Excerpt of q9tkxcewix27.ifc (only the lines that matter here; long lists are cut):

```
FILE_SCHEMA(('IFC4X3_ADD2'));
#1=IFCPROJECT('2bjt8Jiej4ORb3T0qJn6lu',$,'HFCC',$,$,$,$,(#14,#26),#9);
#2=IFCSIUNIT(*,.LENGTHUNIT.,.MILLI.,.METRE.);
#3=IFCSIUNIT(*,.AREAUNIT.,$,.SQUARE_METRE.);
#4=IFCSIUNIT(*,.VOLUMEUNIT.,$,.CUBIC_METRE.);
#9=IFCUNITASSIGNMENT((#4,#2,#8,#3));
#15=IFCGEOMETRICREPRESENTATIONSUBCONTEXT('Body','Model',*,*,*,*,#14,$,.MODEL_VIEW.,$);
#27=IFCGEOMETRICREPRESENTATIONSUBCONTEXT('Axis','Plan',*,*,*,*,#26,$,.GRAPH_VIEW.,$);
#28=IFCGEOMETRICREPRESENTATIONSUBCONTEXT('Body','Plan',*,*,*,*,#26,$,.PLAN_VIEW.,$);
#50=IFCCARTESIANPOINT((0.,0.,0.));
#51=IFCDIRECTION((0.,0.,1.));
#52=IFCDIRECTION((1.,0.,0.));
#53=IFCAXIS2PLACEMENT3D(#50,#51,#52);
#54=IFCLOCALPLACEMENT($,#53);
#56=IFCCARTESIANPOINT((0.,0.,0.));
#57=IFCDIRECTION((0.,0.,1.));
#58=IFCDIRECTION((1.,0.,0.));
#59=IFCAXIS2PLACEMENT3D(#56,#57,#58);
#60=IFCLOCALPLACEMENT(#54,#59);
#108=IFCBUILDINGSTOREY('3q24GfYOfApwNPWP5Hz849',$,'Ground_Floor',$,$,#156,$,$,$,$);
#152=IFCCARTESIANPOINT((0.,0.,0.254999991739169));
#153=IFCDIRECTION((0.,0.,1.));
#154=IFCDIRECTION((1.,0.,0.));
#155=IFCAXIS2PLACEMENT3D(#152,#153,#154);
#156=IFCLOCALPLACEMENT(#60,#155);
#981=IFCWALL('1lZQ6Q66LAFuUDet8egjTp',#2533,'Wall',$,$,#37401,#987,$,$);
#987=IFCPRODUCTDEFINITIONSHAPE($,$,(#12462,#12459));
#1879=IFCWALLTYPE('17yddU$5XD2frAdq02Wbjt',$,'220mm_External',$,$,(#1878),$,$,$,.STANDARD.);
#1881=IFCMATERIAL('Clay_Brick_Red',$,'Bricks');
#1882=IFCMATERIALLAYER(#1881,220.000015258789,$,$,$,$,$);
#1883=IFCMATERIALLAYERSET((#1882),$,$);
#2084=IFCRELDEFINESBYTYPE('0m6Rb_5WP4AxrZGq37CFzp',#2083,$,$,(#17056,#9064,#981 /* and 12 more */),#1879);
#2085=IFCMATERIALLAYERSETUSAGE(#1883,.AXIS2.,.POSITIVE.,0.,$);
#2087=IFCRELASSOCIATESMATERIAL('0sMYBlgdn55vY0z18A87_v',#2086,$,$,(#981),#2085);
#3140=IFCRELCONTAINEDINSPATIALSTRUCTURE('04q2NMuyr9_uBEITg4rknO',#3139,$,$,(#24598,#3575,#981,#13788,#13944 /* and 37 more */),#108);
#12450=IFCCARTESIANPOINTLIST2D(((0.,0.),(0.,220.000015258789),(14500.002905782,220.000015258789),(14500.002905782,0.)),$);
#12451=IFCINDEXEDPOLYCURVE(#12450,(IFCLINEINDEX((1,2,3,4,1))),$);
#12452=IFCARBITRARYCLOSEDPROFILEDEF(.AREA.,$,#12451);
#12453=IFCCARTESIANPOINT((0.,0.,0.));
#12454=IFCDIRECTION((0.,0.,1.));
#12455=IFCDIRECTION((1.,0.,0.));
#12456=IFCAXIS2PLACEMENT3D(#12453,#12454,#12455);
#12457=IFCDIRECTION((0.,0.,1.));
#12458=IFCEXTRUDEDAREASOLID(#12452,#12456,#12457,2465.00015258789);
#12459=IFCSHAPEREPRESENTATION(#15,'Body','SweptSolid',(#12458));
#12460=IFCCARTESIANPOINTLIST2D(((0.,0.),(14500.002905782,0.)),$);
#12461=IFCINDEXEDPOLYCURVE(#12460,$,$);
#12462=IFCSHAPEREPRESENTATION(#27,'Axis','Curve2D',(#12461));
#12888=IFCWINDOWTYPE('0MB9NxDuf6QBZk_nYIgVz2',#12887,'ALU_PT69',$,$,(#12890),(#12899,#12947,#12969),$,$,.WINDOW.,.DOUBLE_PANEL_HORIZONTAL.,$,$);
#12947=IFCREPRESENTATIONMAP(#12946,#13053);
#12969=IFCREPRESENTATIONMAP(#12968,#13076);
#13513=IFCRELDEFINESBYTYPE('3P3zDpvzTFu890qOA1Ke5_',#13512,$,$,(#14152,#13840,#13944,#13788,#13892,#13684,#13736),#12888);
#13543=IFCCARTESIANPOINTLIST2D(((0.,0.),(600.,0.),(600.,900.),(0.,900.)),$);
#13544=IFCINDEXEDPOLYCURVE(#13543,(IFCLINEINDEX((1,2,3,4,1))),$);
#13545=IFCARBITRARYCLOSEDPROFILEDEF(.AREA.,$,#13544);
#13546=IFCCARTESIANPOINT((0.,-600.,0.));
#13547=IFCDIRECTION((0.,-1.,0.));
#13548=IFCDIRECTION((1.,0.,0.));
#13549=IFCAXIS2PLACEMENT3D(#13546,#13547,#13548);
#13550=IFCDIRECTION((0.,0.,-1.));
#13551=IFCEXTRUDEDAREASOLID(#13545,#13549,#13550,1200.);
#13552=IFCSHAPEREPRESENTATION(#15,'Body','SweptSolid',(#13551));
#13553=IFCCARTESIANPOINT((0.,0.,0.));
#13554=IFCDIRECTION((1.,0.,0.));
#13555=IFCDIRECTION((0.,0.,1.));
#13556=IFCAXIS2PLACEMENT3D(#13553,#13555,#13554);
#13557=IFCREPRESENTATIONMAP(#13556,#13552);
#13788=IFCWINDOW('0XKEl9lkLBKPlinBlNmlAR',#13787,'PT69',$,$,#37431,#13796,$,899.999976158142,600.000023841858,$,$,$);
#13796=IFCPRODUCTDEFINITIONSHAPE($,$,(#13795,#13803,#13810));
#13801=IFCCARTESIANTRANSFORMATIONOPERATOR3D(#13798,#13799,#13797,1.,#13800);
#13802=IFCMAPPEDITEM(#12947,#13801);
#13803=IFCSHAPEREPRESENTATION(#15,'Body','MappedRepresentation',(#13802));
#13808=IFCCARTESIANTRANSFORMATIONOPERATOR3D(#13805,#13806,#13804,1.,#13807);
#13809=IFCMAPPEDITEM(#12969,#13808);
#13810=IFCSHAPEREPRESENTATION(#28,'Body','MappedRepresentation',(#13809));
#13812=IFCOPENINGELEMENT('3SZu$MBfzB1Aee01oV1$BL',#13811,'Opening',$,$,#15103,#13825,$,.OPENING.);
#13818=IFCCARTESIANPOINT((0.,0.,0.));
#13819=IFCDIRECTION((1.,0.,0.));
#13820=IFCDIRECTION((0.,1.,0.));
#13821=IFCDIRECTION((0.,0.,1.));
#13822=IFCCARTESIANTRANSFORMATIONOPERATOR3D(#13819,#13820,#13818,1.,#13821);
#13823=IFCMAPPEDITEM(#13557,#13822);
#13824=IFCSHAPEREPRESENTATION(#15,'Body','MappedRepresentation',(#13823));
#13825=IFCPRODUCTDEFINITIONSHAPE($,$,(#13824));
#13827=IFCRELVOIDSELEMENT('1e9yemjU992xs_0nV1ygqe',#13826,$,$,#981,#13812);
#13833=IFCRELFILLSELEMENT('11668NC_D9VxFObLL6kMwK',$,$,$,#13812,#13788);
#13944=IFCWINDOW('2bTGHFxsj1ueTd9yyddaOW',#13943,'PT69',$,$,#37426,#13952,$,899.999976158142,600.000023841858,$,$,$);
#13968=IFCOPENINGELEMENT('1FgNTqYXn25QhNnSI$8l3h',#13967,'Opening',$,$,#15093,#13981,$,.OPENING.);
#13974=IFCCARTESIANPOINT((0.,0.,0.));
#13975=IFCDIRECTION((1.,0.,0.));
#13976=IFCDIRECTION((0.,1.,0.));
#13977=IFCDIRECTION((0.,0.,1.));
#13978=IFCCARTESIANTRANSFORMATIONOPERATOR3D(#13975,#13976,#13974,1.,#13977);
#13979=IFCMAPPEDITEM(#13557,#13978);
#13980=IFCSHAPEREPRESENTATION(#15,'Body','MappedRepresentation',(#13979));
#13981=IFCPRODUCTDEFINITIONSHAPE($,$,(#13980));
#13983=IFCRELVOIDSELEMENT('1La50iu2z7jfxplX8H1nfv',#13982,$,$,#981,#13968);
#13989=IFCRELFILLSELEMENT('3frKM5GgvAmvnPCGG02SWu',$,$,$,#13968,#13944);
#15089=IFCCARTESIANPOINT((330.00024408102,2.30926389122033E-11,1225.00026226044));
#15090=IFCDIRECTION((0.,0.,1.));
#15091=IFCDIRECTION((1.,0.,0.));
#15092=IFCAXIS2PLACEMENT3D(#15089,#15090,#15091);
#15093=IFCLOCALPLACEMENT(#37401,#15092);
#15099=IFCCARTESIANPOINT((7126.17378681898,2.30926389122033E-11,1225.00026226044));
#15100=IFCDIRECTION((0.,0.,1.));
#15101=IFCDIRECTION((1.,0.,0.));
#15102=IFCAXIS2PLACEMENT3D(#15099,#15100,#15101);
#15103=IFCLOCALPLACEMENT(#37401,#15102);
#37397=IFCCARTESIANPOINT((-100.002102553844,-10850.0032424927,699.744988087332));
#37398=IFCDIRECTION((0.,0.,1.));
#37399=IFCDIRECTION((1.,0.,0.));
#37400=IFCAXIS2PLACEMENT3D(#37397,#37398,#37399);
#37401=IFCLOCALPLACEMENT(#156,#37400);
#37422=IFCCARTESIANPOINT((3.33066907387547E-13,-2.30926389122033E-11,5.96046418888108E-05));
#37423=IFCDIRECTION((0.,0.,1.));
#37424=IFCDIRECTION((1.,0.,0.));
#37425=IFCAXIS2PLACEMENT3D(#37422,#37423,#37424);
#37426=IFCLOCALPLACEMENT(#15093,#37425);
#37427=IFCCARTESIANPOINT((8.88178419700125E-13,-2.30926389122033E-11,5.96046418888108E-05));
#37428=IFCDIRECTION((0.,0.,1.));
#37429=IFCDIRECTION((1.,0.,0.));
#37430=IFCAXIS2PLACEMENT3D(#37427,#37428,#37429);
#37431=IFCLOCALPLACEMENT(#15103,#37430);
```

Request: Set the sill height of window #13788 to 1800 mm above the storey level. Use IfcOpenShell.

```python
import numpy as np
import ifcopenshell
import ifcopenshell.api.geometry
import ifcopenshell.geom
import ifcopenshell.util.element
import ifcopenshell.util.placement
import ifcopenshell.util.shape
import ifcopenshell.util.unit

model = ifcopenshell.open("q9tkxcewix27.ifc")
unit_scale = ifcopenshell.util.unit.calculate_unit_scale(model)

window = model.by_guid("0XKEl9lkLBKPlinBlNmlAR")
opening = window.FillsVoids[0].RelatingOpeningElement
storey = ifcopenshell.util.element.get_container(window, ifc_class="IfcBuildingStorey")
level = ifcopenshell.util.placement.get_local_placement(storey.ObjectPlacement)[2, 3]

# The opening's origin need not be at the sill, so measure its lowest point.
shape = ifcopenshell.geom.create_shape(ifcopenshell.geom.settings(), opening)
bottom = ifcopenshell.util.shape.get_shape_bottom_elevation(shape, shape.geometry) / unit_scale
dz = level + 1800.0 - bottom

shift = np.array([0.0, 0.0, dz])
# The window is placed relative to its opening, so it follows when the opening moves.
matrix = ifcopenshell.util.placement.get_local_placement(opening.ObjectPlacement)
matrix[:3, 3] += shift
ifcopenshell.api.geometry.edit_object_placement(
    model, product=opening, matrix=matrix, is_si=False, should_transform_children=True
)

print(f"moved by {dz * unit_scale:+.3f} m")

model.write("q9tkxcewix27-out.ifc")
```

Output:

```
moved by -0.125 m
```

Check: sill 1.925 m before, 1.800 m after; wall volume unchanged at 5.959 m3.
